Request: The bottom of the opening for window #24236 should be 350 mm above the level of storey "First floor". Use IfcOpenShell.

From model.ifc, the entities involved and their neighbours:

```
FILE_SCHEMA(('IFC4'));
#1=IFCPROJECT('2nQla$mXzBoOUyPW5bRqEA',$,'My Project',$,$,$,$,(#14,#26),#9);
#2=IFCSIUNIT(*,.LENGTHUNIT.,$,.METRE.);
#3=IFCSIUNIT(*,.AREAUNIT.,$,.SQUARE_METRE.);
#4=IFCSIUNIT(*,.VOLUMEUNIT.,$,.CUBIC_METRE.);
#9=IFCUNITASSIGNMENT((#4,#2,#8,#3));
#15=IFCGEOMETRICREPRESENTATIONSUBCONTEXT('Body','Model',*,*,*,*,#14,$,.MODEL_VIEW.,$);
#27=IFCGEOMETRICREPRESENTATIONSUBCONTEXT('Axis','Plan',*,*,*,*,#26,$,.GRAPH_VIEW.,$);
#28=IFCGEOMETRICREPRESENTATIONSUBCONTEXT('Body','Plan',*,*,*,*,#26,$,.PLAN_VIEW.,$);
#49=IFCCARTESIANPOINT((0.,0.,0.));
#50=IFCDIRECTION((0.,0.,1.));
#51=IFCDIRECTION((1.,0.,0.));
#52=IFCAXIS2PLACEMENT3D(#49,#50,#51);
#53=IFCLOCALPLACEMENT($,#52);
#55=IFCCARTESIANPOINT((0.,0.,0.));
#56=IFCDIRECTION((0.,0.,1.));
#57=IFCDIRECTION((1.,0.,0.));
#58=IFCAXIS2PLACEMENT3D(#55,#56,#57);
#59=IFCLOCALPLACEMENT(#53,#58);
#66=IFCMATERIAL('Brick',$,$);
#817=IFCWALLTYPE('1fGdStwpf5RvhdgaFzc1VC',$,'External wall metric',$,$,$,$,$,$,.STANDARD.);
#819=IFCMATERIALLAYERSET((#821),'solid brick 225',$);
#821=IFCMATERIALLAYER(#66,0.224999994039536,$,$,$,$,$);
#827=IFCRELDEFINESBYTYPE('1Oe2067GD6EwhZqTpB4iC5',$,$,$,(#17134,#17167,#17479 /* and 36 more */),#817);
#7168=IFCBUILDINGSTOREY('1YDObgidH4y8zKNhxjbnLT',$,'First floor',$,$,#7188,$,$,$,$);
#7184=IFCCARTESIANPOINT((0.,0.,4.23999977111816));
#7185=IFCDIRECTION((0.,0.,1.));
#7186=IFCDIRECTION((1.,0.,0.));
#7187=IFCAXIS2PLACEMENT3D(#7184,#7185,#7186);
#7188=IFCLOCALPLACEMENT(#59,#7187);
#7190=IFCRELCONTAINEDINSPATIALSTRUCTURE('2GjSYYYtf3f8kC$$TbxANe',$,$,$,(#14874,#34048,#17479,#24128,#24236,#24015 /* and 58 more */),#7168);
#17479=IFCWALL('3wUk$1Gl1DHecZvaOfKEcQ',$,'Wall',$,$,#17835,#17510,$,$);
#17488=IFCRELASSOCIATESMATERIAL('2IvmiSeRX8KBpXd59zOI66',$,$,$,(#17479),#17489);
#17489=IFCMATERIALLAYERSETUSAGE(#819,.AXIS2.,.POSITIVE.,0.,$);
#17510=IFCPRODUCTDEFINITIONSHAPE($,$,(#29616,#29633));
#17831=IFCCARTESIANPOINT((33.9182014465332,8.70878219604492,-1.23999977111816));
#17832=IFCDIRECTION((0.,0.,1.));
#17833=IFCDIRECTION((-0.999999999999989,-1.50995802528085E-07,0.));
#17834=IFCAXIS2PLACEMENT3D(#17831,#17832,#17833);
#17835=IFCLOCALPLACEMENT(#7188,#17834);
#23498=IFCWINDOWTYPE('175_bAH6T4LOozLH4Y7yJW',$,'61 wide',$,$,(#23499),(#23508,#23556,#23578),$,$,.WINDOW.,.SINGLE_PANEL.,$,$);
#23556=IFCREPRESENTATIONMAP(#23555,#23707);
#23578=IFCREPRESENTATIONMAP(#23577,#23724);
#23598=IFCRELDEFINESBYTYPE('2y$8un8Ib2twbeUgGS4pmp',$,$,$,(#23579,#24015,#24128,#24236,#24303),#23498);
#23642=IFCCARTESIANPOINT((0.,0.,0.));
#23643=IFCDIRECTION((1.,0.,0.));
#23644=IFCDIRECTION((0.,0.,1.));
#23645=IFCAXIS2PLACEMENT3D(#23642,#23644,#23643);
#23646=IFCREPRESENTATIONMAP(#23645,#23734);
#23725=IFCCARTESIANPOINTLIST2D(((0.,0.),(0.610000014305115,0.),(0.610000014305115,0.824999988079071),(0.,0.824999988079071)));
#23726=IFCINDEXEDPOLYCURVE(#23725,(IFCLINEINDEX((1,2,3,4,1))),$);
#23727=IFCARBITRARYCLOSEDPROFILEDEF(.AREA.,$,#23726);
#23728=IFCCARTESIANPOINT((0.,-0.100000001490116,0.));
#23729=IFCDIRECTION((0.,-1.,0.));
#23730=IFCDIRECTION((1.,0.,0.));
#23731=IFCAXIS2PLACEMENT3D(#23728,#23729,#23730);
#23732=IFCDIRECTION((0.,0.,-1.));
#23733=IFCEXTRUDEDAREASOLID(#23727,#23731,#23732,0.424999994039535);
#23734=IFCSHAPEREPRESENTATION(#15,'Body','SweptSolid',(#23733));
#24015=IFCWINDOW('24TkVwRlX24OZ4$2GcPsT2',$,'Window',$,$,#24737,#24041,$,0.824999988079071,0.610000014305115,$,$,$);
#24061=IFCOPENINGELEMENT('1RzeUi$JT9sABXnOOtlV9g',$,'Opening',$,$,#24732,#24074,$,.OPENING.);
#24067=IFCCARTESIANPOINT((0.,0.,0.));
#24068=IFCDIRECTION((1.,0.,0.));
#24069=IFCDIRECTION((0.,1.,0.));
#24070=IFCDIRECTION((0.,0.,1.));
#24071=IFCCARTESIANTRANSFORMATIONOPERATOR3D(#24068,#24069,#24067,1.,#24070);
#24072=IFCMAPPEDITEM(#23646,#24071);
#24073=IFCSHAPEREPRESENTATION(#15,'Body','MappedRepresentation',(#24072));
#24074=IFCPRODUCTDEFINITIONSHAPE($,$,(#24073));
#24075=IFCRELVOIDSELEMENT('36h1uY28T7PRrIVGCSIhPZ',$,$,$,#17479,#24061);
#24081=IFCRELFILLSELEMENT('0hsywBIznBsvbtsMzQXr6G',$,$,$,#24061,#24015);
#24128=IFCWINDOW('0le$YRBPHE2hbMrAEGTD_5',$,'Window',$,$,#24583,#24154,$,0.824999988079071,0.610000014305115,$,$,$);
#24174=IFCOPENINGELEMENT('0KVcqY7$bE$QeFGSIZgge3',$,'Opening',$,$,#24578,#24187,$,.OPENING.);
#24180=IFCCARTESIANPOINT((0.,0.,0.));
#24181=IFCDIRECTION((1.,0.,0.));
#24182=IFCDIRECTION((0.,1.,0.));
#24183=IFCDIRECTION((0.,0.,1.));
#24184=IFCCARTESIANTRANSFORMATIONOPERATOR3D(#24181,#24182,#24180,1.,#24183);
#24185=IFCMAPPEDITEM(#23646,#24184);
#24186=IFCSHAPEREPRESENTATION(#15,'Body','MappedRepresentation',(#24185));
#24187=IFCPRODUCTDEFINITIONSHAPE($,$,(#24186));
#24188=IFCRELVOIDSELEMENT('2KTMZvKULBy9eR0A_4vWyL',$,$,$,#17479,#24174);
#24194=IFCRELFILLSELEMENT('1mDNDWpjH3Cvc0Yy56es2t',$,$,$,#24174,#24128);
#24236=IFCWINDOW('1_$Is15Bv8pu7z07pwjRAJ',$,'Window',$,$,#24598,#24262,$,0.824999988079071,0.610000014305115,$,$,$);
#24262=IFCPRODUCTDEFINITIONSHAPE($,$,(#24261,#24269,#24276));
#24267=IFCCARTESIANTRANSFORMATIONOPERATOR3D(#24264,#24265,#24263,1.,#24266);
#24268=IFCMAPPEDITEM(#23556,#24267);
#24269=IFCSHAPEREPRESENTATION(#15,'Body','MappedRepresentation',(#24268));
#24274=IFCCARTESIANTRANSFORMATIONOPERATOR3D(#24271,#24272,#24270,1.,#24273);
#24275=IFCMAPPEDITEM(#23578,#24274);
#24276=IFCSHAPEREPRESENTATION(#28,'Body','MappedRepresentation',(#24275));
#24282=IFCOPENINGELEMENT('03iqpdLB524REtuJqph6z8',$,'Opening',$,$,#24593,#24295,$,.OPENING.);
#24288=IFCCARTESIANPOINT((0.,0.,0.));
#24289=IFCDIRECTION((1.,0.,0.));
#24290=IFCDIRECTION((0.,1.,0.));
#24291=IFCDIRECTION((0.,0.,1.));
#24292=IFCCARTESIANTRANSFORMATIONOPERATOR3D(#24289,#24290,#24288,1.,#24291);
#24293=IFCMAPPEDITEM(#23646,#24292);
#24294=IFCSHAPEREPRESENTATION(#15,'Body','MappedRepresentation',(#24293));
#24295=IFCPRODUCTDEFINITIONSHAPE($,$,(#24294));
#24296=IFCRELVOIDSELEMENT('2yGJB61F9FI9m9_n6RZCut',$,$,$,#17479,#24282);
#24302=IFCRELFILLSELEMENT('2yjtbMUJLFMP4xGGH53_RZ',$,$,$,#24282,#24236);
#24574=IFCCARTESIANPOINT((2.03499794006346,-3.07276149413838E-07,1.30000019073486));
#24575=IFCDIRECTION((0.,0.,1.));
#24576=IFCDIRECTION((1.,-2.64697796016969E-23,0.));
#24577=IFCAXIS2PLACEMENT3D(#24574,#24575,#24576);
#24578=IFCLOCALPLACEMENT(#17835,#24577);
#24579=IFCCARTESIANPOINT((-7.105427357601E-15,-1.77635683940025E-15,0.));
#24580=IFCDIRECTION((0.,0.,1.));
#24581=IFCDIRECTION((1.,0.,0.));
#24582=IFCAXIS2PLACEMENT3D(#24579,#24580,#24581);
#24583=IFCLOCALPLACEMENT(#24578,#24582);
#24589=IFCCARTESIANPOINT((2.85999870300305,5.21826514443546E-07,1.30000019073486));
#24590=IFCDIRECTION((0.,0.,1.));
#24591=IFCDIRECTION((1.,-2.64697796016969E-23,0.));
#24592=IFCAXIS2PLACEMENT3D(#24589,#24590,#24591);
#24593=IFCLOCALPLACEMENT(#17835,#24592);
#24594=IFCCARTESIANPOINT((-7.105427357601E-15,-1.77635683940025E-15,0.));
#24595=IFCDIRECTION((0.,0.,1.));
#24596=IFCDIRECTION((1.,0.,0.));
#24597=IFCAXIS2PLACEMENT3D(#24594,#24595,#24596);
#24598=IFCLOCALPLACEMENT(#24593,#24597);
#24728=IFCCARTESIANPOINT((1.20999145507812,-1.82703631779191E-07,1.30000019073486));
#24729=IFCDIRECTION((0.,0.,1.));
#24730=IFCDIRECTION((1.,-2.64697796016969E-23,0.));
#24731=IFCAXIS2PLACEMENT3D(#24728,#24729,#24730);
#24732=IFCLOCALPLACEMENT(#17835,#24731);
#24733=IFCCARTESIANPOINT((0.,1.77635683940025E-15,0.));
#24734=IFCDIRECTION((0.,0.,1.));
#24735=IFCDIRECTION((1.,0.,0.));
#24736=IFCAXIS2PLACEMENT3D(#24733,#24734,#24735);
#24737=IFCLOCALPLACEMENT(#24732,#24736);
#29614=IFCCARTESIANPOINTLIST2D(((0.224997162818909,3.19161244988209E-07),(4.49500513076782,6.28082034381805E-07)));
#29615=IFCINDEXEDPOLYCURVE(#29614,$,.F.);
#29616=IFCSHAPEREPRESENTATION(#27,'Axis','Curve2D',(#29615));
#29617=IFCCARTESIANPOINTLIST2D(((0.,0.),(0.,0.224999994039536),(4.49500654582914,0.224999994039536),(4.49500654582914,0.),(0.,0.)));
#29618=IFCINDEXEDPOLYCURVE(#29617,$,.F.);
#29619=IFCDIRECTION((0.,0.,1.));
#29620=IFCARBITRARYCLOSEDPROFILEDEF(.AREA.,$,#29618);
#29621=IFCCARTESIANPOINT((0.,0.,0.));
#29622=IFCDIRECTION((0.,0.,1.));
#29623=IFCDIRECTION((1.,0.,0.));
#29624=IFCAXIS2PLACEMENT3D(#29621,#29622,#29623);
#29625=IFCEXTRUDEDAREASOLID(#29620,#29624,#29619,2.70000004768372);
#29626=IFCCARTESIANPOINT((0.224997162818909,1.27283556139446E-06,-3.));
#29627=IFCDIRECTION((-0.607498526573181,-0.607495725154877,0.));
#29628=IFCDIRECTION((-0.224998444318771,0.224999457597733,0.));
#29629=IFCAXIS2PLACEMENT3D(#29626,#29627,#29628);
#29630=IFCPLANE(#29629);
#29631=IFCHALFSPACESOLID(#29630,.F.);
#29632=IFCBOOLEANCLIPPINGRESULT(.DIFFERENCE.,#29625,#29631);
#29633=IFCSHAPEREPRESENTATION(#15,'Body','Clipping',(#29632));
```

```python
import numpy as np
import ifcopenshell
import ifcopenshell.api.geometry
import ifcopenshell.geom
import ifcopenshell.util.element
import ifcopenshell.util.placement
import ifcopenshell.util.shape
import ifcopenshell.util.unit

model = ifcopenshell.open("model.ifc")
unit_scale = ifcopenshell.util.unit.calculate_unit_scale(model)

window = model.by_id(24236)
opening = window.FillsVoids[0].RelatingOpeningElement
storey = ifcopenshell.util.element.get_container(window, ifc_class="IfcBuildingStorey")
level = ifcopenshell.util.placement.get_local_placement(storey.ObjectPlacement)[2, 3]

# The opening's origin need not be at the sill, so measure its lowest point.
shape = ifcopenshell.geom.create_shape(ifcopenshell.geom.settings(), opening)
bottom = ifcopenshell.util.shape.get_shape_bottom_elevation(shape, shape.geometry) / unit_scale
dz = level + 0.35 / unit_scale - bottom

shift = np.array([0.0, 0.0, dz])
# The window is placed relative to its opening, so it follows when the opening moves.
matrix = ifcopenshell.util.placement.get_local_placement(opening.ObjectPlacement)
matrix[:3, 3] += shift
ifcopenshell.api.geometry.edit_object_placement(
    model, product=opening, matrix=matrix, is_si=False, should_transform_children=True
)

print(f"moved by {dz * unit_scale:+.3f} m")

model.write("model_edited.ifc")
```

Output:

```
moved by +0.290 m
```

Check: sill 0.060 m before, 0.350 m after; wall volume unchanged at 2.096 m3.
